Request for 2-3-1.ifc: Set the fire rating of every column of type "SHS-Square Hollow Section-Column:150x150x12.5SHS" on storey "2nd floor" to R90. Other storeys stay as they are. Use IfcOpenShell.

First a look at what the model holds.

```python
import ifcopenshell
import ifcopenshell.util.element

model = ifcopenshell.open("2-3-1.ifc")
print(model.schema)
storey = next(s for s in model.by_type("IfcBuildingStorey") if s.Name == "2nd floor")
columns = [e for e in ifcopenshell.util.element.get_decomposition(storey) if e.is_a("IfcColumn")]
seen = {}
for e in columns:
    element_type = ifcopenshell.util.element.get_type(e)
    key = (element_type.Name if element_type != e and element_type else None, ifcopenshell.util.element.get_pset(e, "Pset_ColumnCommon", "FireRating"))
    seen[key] = seen.get(key, 0) + 1
for (name, value), count in sorted(seen.items(), key=str):
    print(count, "x", name, "|", value)
```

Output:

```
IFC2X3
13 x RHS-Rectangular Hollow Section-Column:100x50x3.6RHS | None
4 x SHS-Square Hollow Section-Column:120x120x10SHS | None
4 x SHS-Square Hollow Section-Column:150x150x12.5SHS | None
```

```python
import ifcopenshell
import ifcopenshell.api.pset
import ifcopenshell.util.element

model = ifcopenshell.open("2-3-1.ifc")

storey = next(s for s in model.by_type("IfcBuildingStorey") if s.Name == "2nd floor")
columns = [e for e in ifcopenshell.util.element.get_decomposition(storey) if e.is_a("IfcColumn")]

count = 0
for e in columns:
    element_type = ifcopenshell.util.element.get_type(e)
    if element_type in (None, e) or element_type.Name != "SHS-Square Hollow Section-Column:150x150x12.5SHS":
        continue
    # add_pset returns the element's existing set when there is one.
    pset = ifcopenshell.api.pset.add_pset(model, product=e, name="Pset_ColumnCommon")
    ifcopenshell.api.pset.edit_pset(model, pset=pset, properties={"FireRating": "R90"})
    count += 1

print(count, "columns updated")

model.write("2-3-1_edited.ifc")
```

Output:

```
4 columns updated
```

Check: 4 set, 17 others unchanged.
